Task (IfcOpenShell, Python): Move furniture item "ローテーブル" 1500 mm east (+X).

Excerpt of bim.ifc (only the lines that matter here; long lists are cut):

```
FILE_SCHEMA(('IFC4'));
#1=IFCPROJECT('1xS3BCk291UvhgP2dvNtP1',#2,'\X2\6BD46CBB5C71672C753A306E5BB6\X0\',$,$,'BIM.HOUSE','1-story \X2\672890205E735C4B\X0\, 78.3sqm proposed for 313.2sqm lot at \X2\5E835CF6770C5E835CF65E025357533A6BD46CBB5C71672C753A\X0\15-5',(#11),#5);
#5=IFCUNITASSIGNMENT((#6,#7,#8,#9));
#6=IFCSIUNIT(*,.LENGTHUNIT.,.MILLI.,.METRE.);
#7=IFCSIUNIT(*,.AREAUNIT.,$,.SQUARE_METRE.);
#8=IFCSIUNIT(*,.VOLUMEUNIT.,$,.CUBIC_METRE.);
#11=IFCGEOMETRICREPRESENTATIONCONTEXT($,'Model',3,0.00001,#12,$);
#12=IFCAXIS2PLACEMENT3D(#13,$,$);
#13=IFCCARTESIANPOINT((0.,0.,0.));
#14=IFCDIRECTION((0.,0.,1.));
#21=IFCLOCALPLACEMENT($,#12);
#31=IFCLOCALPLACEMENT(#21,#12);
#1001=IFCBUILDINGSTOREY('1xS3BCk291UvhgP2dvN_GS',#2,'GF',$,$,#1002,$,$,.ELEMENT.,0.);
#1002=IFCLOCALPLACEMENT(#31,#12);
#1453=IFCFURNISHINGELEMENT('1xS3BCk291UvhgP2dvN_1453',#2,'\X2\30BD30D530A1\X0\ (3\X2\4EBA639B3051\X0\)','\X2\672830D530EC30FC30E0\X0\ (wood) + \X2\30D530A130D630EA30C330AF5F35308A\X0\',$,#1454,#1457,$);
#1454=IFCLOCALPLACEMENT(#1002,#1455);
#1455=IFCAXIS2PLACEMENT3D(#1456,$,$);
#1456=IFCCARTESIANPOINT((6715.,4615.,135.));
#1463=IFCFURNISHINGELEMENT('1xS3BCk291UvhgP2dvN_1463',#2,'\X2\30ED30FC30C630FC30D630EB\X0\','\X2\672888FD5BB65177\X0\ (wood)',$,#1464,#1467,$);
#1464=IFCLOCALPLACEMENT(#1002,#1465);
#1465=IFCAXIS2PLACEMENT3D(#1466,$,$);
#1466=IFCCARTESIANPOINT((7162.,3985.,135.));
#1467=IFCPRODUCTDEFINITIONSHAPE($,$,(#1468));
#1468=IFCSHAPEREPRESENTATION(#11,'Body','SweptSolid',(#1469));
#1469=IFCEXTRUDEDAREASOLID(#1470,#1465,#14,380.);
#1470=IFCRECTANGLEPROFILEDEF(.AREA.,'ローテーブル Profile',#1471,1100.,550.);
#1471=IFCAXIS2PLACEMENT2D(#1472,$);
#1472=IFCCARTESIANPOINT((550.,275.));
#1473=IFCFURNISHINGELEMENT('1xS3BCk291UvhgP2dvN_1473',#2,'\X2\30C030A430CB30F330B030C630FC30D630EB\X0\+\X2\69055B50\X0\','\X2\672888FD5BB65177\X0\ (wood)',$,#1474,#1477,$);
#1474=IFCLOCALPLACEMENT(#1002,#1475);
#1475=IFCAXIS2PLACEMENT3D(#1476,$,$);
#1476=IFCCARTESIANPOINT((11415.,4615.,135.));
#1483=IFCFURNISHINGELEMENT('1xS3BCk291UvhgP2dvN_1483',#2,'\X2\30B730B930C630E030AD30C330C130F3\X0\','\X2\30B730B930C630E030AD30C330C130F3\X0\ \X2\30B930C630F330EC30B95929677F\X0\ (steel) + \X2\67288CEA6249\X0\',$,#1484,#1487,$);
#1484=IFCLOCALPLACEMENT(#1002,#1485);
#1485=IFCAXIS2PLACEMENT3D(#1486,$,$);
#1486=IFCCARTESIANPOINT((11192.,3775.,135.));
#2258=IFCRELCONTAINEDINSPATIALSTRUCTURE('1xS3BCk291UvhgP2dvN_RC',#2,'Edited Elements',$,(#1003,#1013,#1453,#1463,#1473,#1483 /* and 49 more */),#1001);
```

```python
import ifcopenshell
import ifcopenshell.api.geometry
import ifcopenshell.util.placement
import ifcopenshell.util.unit

model = ifcopenshell.open("bim.ifc")
unit_scale = ifcopenshell.util.unit.calculate_unit_scale(model)

item = model.by_guid("1xS3BCk291UvhgP2dvN_1463")
matrix = ifcopenshell.util.placement.get_local_placement(item.ObjectPlacement)
matrix[0, 3] += 1.5 / unit_scale
ifcopenshell.api.geometry.edit_object_placement(model, product=item, matrix=matrix, is_si=False)

print(ifcopenshell.util.placement.get_local_placement(item.ObjectPlacement).round(3) + 0.0)

model.write("bim_edited.ifc")
```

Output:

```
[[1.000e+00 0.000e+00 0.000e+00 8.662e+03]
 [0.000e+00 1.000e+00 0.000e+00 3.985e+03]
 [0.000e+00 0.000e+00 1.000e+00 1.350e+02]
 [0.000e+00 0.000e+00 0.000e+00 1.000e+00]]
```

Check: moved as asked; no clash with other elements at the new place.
